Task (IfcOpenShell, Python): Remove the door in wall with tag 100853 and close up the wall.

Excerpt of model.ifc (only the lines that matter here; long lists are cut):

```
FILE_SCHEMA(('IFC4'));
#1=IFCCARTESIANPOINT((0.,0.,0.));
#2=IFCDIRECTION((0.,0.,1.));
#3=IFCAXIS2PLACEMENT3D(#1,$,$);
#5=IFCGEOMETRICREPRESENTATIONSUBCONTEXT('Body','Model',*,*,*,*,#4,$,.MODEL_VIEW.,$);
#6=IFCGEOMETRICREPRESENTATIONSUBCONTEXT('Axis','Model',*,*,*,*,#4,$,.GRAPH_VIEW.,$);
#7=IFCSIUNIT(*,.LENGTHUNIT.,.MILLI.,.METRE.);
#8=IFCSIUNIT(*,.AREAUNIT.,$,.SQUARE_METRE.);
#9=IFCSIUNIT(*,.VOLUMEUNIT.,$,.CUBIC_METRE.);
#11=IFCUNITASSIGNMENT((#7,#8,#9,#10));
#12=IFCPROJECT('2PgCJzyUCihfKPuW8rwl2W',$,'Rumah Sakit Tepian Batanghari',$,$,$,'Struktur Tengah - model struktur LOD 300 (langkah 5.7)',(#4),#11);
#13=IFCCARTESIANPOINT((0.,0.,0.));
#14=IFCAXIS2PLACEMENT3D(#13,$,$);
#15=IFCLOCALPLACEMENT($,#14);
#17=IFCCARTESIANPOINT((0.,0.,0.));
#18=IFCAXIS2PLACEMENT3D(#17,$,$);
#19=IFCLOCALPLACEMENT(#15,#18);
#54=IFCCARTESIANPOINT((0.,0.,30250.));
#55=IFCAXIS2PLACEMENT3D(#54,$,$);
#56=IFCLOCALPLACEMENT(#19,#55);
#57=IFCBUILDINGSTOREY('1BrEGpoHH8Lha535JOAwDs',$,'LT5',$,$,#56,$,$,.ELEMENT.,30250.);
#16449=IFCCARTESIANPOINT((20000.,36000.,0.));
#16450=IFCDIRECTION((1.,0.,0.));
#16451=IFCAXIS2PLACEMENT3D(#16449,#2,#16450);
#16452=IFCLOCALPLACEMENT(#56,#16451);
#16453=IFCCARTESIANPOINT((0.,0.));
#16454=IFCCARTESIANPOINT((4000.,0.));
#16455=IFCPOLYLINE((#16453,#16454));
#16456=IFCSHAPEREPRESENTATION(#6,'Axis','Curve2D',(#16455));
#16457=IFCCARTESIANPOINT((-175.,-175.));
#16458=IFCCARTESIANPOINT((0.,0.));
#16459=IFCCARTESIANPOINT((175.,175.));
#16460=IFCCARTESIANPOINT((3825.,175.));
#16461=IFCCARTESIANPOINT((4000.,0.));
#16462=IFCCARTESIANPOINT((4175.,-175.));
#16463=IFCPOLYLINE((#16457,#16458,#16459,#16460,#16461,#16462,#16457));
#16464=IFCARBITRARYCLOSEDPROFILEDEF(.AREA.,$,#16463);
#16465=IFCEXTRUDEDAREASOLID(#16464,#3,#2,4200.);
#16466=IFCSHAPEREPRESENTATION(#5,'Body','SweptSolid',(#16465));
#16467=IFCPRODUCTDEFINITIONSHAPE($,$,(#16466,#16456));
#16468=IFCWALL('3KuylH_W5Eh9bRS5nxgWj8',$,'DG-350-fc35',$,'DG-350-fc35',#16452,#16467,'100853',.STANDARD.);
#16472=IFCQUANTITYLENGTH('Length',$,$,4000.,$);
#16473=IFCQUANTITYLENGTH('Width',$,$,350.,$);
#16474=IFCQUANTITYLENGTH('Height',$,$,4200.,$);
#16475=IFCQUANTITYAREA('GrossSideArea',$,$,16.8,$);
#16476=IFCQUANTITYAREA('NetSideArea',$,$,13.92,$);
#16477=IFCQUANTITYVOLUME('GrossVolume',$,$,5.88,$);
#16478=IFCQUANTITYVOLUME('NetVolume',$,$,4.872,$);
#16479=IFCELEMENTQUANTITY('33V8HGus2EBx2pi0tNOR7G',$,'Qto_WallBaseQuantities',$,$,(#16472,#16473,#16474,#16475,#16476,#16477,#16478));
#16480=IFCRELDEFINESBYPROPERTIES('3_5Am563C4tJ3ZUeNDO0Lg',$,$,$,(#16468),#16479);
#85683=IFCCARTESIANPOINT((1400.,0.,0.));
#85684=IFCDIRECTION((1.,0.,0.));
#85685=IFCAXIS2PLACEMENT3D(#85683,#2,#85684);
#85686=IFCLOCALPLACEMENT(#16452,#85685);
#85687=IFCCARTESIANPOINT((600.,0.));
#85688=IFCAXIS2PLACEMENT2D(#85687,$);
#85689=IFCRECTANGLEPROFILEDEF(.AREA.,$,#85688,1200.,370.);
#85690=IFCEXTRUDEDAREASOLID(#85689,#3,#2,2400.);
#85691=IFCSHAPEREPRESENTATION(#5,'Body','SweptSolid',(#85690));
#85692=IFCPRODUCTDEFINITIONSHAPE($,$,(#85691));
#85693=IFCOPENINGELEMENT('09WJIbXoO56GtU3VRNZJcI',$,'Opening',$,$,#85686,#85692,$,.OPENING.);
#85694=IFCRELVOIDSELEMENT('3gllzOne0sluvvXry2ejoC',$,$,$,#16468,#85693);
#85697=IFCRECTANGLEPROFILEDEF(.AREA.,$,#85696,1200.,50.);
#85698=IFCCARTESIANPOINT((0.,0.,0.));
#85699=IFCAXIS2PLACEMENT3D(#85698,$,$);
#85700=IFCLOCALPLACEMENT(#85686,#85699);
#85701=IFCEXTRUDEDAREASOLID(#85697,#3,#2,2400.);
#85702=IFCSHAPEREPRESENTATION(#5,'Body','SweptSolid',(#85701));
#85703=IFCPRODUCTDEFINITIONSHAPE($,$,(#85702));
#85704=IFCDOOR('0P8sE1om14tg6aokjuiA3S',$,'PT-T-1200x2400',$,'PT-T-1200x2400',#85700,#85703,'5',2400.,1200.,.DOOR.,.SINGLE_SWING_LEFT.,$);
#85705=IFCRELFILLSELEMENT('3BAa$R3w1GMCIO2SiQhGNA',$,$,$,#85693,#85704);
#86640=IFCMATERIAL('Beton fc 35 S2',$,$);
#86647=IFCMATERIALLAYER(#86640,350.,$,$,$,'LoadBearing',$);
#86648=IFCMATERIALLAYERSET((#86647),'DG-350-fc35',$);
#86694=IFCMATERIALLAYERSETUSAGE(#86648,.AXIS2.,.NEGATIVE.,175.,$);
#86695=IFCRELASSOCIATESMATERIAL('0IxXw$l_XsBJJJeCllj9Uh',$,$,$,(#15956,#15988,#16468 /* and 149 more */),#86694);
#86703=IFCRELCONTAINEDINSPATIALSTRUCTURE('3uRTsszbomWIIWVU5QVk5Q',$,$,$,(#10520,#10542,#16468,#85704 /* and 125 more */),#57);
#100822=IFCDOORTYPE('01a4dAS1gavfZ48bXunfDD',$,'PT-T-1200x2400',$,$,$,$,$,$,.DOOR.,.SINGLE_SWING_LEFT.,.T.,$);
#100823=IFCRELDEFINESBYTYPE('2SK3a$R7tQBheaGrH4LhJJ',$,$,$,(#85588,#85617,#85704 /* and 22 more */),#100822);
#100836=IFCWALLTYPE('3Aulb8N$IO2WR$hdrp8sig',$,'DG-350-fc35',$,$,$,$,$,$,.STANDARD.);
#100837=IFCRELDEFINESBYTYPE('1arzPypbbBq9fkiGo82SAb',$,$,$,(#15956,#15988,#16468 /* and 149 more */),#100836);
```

```python
import ifcopenshell
import ifcopenshell.api.feature
import ifcopenshell.api.pset
import ifcopenshell.api.root
import ifcopenshell.geom
import ifcopenshell.util.element
import ifcopenshell.util.shape
import ifcopenshell.util.unit

model = ifcopenshell.open("model.ifc")
area_scale = ifcopenshell.util.unit.calculate_unit_scale(model, "AREAUNIT")
volume_scale = ifcopenshell.util.unit.calculate_unit_scale(model, "VOLUMEUNIT")
settings = ifcopenshell.geom.settings()


def volume(element):
    """Net volume in cubic metres, openings subtracted."""
    shape = ifcopenshell.geom.create_shape(settings, element)
    return ifcopenshell.util.shape.get_volume(shape.geometry)


door = model.by_id(85704)
opening = door.FillsVoids[0].RelatingOpeningElement
wall = opening.VoidsElements[0].RelatingBuildingElement
before = volume(wall)

ifcopenshell.api.root.remove_product(model, product=door)
ifcopenshell.api.feature.remove_feature(model, feature=opening)

after = volume(wall)
thickness = 0.35  # wall thickness in metres

# Update the wall's stored quantities.
qto = model.by_id(ifcopenshell.util.element.get_pset(wall, "Qto_WallBaseQuantities", should_inherit=False)["id"])
ifcopenshell.api.pset.edit_qto(model, qto=qto, properties={
    "NetSideArea": after / thickness / area_scale,
    "NetVolume": after / volume_scale,
})

print(f"wall volume {before:.3f} -> {after:.3f} m3")

model.write("model_v2.ifc")
```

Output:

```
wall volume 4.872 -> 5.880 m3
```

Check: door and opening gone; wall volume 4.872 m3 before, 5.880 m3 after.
